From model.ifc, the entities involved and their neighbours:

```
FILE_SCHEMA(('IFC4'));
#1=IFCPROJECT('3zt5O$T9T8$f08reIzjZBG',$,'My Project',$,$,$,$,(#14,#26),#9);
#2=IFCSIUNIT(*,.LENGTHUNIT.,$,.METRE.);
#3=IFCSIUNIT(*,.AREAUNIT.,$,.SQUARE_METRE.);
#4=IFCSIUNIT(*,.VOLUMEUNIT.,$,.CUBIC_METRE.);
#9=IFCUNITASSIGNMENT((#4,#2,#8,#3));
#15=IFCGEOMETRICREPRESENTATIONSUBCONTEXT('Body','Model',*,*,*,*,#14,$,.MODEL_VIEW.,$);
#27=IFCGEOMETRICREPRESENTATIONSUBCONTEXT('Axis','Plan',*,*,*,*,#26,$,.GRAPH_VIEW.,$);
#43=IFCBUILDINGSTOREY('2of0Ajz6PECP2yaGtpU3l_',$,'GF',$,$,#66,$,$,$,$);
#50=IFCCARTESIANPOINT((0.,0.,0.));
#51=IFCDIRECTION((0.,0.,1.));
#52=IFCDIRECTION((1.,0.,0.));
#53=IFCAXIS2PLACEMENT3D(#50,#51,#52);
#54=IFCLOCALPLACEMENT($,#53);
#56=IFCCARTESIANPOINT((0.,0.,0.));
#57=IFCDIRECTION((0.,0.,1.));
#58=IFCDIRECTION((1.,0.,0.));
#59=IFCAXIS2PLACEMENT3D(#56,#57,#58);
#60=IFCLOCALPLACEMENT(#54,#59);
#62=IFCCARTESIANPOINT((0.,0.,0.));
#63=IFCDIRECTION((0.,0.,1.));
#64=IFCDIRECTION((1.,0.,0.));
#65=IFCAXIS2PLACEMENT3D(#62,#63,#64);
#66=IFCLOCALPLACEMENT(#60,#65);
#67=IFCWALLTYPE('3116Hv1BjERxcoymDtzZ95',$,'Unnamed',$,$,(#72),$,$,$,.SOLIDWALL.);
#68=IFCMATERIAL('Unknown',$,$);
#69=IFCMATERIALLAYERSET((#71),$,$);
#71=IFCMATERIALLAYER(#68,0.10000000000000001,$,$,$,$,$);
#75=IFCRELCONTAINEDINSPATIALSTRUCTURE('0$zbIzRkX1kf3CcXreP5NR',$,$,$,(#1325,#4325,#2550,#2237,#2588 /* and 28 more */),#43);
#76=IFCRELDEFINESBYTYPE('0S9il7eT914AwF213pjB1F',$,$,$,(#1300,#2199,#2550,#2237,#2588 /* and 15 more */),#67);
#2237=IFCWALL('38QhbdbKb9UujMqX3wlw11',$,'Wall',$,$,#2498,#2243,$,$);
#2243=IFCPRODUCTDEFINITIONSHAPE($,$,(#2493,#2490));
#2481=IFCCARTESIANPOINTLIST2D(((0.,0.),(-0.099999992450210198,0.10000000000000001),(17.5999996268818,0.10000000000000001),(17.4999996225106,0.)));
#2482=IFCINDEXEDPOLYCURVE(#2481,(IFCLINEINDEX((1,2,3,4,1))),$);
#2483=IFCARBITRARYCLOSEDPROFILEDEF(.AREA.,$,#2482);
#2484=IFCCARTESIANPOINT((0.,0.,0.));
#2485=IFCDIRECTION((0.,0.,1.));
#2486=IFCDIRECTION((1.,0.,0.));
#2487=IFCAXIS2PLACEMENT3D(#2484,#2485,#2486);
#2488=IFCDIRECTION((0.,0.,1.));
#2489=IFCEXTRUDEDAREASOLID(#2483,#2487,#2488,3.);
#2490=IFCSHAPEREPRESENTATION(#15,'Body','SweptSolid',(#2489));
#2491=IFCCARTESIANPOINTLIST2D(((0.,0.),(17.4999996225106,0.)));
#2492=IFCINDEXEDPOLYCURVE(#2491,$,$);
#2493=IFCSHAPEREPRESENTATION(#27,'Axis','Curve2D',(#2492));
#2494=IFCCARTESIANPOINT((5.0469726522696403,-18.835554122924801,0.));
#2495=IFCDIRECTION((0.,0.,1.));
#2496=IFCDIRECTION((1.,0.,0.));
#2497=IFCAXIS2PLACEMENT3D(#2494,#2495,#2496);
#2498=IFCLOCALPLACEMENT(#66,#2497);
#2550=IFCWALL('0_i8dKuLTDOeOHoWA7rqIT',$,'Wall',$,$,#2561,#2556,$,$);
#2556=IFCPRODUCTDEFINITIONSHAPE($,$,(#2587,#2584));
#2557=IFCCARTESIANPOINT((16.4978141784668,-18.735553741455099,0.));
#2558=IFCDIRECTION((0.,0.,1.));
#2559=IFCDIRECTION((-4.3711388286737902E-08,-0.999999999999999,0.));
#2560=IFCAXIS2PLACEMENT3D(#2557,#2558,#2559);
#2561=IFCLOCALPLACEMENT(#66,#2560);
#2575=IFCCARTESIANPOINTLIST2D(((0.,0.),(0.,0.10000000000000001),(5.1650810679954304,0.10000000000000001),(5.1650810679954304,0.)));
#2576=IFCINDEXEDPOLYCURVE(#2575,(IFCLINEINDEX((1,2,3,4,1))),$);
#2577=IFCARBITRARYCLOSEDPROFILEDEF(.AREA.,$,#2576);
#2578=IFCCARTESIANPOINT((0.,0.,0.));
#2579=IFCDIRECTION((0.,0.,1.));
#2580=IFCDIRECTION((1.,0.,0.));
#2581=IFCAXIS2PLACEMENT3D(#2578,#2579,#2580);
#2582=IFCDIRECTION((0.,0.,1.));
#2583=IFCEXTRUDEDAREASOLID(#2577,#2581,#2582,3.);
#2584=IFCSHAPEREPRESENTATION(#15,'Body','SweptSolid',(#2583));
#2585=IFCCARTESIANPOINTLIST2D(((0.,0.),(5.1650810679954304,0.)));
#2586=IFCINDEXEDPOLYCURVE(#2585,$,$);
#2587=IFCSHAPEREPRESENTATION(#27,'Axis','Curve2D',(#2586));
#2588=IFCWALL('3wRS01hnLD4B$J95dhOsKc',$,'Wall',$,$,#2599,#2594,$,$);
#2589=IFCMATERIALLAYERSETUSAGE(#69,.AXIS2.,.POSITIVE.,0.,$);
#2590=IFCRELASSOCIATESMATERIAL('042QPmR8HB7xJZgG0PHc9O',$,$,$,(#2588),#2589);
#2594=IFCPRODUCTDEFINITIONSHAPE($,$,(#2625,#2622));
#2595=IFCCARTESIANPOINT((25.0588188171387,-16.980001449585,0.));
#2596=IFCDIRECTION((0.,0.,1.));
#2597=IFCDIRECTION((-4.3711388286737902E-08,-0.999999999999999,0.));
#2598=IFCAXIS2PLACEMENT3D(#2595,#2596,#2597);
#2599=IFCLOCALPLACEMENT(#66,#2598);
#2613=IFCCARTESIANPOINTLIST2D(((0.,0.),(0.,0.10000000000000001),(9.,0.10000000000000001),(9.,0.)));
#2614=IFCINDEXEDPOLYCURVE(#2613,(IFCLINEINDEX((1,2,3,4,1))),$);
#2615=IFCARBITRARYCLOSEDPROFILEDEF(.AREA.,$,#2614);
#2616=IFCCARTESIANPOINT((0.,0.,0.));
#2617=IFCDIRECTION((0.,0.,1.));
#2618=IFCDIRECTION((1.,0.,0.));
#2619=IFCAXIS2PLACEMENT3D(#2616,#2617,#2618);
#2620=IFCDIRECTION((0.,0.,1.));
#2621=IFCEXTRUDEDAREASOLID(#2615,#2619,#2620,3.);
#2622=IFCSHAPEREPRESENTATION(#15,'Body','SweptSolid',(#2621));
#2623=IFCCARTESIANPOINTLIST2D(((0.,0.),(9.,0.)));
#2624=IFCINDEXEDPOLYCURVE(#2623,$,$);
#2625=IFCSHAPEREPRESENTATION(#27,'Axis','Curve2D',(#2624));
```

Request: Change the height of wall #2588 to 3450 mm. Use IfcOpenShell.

```python
import ifcopenshell
import ifcopenshell.geom
import ifcopenshell.util.representation
import ifcopenshell.util.shape
import ifcopenshell.util.unit

model = ifcopenshell.open("model.ifc")
unit_scale = ifcopenshell.util.unit.calculate_unit_scale(model)
settings = ifcopenshell.geom.settings()


def volume(element):
    """Net volume in cubic metres, openings subtracted."""
    shape = ifcopenshell.geom.create_shape(settings, element)
    return ifcopenshell.util.shape.get_volume(shape.geometry)


wall = model.by_guid("3wRS01hnLD4B$J95dhOsKc")
before = volume(wall)

body = ifcopenshell.util.representation.get_representation(wall, "Model", "Body")
solid = body.Items[0]
old_height = solid.Depth
solid.Depth = 3.45 / unit_scale
after = volume(wall)

print(f"height {old_height:g} -> {solid.Depth:g}, volume {before:.3f} -> {after:.3f} m3")

model.write("model_v2.ifc")
```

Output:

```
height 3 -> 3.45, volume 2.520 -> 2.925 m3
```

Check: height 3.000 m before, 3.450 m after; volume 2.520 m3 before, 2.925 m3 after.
